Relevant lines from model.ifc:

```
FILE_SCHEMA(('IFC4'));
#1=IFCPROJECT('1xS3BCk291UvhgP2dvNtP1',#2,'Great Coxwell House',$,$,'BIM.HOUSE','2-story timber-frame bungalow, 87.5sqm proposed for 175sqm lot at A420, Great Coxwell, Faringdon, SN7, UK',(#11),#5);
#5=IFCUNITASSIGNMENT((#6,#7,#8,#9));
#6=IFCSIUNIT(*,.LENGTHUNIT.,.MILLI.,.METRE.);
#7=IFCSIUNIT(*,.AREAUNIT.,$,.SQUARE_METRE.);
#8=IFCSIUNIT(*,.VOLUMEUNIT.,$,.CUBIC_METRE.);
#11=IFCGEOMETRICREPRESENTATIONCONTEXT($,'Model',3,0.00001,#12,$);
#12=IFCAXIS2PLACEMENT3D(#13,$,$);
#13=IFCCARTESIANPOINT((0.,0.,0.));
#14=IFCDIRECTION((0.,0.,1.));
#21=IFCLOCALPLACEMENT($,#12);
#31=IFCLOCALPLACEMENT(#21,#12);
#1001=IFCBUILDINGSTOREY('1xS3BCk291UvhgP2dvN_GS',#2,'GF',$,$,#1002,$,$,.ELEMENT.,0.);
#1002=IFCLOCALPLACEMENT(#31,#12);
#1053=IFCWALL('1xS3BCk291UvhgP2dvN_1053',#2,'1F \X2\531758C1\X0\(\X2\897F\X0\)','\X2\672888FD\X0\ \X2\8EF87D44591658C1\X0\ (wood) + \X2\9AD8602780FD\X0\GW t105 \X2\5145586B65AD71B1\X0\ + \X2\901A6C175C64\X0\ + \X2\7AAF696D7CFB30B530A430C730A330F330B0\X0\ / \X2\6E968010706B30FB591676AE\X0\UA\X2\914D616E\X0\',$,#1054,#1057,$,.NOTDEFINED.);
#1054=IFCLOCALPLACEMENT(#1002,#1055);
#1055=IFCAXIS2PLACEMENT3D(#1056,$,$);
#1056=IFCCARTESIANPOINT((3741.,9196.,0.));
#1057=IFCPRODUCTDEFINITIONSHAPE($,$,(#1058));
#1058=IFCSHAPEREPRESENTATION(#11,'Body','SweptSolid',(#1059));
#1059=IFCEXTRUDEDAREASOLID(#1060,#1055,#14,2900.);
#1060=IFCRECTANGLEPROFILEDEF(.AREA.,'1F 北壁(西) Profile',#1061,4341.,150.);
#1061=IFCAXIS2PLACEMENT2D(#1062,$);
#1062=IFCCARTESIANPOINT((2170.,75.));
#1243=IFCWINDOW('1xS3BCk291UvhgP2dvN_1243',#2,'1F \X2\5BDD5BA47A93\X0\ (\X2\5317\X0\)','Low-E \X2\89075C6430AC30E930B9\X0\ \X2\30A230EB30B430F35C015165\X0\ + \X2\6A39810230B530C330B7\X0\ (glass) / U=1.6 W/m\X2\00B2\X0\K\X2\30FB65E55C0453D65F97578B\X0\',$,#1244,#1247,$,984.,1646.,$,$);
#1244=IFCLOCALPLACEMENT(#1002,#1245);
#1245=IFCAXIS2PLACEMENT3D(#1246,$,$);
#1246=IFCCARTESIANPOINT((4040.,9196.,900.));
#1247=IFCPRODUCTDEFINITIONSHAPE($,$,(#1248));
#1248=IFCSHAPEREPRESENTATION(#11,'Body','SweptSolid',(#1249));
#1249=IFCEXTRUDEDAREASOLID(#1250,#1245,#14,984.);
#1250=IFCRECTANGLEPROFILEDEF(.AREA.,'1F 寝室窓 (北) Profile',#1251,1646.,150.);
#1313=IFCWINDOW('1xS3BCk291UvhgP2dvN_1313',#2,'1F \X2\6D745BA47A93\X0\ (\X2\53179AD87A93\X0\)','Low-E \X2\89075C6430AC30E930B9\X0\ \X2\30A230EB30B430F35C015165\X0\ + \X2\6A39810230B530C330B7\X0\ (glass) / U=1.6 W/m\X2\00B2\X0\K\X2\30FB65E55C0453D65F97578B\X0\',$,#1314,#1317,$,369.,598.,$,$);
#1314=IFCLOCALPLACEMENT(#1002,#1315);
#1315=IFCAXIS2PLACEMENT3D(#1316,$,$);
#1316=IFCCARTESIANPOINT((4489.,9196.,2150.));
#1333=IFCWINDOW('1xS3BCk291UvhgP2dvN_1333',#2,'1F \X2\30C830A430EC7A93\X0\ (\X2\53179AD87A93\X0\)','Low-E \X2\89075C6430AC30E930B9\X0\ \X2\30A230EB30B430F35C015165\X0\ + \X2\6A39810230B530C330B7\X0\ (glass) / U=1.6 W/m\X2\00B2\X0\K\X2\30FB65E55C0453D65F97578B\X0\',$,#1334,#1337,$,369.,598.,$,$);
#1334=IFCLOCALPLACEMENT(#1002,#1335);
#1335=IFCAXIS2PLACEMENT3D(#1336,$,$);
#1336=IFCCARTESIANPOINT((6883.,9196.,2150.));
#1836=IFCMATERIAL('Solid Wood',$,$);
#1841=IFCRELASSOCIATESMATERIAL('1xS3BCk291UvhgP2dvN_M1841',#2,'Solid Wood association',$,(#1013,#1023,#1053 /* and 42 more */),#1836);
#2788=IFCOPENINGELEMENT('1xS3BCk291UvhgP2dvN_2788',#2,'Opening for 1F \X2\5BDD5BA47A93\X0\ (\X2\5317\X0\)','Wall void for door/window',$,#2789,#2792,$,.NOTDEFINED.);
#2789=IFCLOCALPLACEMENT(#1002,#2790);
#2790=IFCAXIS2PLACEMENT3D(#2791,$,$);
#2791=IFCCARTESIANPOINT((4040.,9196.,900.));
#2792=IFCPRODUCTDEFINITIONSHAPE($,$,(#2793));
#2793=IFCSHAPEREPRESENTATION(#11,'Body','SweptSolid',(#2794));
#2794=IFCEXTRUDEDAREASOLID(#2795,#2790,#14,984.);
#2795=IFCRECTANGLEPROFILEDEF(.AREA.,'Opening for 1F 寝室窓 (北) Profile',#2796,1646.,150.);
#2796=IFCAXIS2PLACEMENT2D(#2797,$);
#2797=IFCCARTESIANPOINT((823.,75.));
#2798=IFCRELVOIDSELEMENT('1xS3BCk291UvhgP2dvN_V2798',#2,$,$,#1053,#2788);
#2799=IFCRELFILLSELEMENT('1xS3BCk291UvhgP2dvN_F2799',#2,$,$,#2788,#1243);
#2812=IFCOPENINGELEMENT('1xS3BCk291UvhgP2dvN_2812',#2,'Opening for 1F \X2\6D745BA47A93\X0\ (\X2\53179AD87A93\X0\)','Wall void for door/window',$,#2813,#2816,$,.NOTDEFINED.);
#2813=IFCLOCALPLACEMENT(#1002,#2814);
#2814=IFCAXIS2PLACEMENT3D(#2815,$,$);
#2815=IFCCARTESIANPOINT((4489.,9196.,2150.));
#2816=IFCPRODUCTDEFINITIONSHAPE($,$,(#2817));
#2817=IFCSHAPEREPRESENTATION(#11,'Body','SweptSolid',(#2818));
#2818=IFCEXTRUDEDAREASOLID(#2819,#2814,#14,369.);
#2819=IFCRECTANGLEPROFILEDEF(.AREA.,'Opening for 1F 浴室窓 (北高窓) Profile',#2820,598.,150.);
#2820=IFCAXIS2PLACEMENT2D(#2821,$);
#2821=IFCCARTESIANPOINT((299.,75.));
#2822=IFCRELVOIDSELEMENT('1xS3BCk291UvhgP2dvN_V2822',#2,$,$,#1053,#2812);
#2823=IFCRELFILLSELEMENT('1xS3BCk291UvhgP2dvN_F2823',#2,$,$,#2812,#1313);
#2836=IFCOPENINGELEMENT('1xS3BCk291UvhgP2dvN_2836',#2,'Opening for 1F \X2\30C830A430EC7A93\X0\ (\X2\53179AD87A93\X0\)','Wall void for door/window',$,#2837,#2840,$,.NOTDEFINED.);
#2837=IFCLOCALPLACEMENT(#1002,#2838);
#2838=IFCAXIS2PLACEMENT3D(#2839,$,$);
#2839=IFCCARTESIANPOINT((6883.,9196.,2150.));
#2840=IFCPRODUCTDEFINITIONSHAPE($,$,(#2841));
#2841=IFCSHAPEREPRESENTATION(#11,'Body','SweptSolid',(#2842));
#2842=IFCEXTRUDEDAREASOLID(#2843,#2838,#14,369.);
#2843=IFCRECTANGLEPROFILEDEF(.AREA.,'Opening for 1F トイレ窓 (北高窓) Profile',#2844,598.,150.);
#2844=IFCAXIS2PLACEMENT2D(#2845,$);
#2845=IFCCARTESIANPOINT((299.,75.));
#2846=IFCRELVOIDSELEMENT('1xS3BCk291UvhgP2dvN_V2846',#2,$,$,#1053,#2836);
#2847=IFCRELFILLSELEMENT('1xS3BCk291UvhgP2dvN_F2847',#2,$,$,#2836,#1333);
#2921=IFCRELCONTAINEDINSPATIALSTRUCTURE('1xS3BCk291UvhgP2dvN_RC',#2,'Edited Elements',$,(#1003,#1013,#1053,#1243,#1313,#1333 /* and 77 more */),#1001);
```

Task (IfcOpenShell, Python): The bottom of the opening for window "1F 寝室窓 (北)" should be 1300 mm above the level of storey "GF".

```python
import numpy as np
import ifcopenshell
import ifcopenshell.api.geometry
import ifcopenshell.geom
import ifcopenshell.util.element
import ifcopenshell.util.placement
import ifcopenshell.util.shape
import ifcopenshell.util.unit

model = ifcopenshell.open("model.ifc")
unit_scale = ifcopenshell.util.unit.calculate_unit_scale(model)

window = model.by_guid("1xS3BCk291UvhgP2dvN_1243")
opening = window.FillsVoids[0].RelatingOpeningElement
storey = ifcopenshell.util.element.get_container(window, ifc_class="IfcBuildingStorey")
level = ifcopenshell.util.placement.get_local_placement(storey.ObjectPlacement)[2, 3]

# The opening's origin need not be at the sill, so measure its lowest point.
shape = ifcopenshell.geom.create_shape(ifcopenshell.geom.settings(), opening)
bottom = ifcopenshell.util.shape.get_shape_bottom_elevation(shape, shape.geometry) / unit_scale
dz = level + 1.3 / unit_scale - bottom

shift = np.array([0.0, 0.0, dz])
# The window is not placed relative to its opening, so move both.
for product in (opening, window):
    matrix = ifcopenshell.util.placement.get_local_placement(product.ObjectPlacement)
    matrix[:3, 3] += shift
    ifcopenshell.api.geometry.edit_object_placement(model, product=product, matrix=matrix, is_si=False)

print(f"moved by {dz * unit_scale:+.3f} m")

model.write("model_edited.ifc")
```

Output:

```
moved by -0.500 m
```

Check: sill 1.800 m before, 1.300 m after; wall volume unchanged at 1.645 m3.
